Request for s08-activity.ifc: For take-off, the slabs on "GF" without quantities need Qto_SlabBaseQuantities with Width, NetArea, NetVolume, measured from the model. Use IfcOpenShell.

First a look at what the model holds.

```python
import ifcopenshell
import ifcopenshell.util.element
import ifcopenshell.util.unit

model = ifcopenshell.open("s08-activity.ifc")
print(model.schema)
for unit_type in ("LENGTHUNIT", "AREAUNIT", "VOLUMEUNIT"):
    print(unit_type, ifcopenshell.util.unit.calculate_unit_scale(model, unit_type))
storey = next(s for s in model.by_type("IfcBuildingStorey") if s.Name == "GF")
slabs = [e for e in ifcopenshell.util.element.get_decomposition(storey) if e.is_a("IfcSlab")]
for e in sorted(slabs, key=lambda e: e.id()):
    print(e.id(), e.is_a(), e.Name, list(ifcopenshell.util.element.get_psets(e, qtos_only=True)), sep=" | ")
```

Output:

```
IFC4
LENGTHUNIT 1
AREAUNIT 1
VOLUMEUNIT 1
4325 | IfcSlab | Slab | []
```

```python
import ifcopenshell
import ifcopenshell.api.pset
import ifcopenshell.geom
import ifcopenshell.util.element
import ifcopenshell.util.shape
import ifcopenshell.util.unit

model = ifcopenshell.open("s08-activity.ifc")
unit_scale = ifcopenshell.util.unit.calculate_unit_scale(model)
area_scale = ifcopenshell.util.unit.calculate_unit_scale(model, "AREAUNIT")
volume_scale = ifcopenshell.util.unit.calculate_unit_scale(model, "VOLUMEUNIT")
settings = ifcopenshell.geom.settings()

storey = next(s for s in model.by_type("IfcBuildingStorey") if s.Name == "GF")
slabs = [e for e in ifcopenshell.util.element.get_decomposition(storey) if e.is_a("IfcSlab")]

for e in sorted(slabs, key=lambda e: e.id()):
    if ifcopenshell.util.element.get_psets(e, qtos_only=True, should_inherit=False):
        continue
    # Geometry comes back in metres, in the element's own axes.
    shape = ifcopenshell.geom.create_shape(settings, e)
    values = {
        "Width": ifcopenshell.util.shape.get_z(shape.geometry) / unit_scale,
        "NetArea": ifcopenshell.util.shape.get_footprint_area(shape.geometry) / area_scale,
        "NetVolume": ifcopenshell.util.shape.get_volume(shape.geometry) / volume_scale,
    }
    qto = ifcopenshell.api.pset.add_qto(model, product=e, name="Qto_SlabBaseQuantities")
    ifcopenshell.api.pset.edit_qto(model, qto=qto, properties=values)
    print(e.id(), {k: round(v, 3) for k, v in values.items()})

model.write("s08-activity_v2.ifc")
```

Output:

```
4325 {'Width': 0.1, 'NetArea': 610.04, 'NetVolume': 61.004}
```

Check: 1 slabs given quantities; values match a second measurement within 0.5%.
